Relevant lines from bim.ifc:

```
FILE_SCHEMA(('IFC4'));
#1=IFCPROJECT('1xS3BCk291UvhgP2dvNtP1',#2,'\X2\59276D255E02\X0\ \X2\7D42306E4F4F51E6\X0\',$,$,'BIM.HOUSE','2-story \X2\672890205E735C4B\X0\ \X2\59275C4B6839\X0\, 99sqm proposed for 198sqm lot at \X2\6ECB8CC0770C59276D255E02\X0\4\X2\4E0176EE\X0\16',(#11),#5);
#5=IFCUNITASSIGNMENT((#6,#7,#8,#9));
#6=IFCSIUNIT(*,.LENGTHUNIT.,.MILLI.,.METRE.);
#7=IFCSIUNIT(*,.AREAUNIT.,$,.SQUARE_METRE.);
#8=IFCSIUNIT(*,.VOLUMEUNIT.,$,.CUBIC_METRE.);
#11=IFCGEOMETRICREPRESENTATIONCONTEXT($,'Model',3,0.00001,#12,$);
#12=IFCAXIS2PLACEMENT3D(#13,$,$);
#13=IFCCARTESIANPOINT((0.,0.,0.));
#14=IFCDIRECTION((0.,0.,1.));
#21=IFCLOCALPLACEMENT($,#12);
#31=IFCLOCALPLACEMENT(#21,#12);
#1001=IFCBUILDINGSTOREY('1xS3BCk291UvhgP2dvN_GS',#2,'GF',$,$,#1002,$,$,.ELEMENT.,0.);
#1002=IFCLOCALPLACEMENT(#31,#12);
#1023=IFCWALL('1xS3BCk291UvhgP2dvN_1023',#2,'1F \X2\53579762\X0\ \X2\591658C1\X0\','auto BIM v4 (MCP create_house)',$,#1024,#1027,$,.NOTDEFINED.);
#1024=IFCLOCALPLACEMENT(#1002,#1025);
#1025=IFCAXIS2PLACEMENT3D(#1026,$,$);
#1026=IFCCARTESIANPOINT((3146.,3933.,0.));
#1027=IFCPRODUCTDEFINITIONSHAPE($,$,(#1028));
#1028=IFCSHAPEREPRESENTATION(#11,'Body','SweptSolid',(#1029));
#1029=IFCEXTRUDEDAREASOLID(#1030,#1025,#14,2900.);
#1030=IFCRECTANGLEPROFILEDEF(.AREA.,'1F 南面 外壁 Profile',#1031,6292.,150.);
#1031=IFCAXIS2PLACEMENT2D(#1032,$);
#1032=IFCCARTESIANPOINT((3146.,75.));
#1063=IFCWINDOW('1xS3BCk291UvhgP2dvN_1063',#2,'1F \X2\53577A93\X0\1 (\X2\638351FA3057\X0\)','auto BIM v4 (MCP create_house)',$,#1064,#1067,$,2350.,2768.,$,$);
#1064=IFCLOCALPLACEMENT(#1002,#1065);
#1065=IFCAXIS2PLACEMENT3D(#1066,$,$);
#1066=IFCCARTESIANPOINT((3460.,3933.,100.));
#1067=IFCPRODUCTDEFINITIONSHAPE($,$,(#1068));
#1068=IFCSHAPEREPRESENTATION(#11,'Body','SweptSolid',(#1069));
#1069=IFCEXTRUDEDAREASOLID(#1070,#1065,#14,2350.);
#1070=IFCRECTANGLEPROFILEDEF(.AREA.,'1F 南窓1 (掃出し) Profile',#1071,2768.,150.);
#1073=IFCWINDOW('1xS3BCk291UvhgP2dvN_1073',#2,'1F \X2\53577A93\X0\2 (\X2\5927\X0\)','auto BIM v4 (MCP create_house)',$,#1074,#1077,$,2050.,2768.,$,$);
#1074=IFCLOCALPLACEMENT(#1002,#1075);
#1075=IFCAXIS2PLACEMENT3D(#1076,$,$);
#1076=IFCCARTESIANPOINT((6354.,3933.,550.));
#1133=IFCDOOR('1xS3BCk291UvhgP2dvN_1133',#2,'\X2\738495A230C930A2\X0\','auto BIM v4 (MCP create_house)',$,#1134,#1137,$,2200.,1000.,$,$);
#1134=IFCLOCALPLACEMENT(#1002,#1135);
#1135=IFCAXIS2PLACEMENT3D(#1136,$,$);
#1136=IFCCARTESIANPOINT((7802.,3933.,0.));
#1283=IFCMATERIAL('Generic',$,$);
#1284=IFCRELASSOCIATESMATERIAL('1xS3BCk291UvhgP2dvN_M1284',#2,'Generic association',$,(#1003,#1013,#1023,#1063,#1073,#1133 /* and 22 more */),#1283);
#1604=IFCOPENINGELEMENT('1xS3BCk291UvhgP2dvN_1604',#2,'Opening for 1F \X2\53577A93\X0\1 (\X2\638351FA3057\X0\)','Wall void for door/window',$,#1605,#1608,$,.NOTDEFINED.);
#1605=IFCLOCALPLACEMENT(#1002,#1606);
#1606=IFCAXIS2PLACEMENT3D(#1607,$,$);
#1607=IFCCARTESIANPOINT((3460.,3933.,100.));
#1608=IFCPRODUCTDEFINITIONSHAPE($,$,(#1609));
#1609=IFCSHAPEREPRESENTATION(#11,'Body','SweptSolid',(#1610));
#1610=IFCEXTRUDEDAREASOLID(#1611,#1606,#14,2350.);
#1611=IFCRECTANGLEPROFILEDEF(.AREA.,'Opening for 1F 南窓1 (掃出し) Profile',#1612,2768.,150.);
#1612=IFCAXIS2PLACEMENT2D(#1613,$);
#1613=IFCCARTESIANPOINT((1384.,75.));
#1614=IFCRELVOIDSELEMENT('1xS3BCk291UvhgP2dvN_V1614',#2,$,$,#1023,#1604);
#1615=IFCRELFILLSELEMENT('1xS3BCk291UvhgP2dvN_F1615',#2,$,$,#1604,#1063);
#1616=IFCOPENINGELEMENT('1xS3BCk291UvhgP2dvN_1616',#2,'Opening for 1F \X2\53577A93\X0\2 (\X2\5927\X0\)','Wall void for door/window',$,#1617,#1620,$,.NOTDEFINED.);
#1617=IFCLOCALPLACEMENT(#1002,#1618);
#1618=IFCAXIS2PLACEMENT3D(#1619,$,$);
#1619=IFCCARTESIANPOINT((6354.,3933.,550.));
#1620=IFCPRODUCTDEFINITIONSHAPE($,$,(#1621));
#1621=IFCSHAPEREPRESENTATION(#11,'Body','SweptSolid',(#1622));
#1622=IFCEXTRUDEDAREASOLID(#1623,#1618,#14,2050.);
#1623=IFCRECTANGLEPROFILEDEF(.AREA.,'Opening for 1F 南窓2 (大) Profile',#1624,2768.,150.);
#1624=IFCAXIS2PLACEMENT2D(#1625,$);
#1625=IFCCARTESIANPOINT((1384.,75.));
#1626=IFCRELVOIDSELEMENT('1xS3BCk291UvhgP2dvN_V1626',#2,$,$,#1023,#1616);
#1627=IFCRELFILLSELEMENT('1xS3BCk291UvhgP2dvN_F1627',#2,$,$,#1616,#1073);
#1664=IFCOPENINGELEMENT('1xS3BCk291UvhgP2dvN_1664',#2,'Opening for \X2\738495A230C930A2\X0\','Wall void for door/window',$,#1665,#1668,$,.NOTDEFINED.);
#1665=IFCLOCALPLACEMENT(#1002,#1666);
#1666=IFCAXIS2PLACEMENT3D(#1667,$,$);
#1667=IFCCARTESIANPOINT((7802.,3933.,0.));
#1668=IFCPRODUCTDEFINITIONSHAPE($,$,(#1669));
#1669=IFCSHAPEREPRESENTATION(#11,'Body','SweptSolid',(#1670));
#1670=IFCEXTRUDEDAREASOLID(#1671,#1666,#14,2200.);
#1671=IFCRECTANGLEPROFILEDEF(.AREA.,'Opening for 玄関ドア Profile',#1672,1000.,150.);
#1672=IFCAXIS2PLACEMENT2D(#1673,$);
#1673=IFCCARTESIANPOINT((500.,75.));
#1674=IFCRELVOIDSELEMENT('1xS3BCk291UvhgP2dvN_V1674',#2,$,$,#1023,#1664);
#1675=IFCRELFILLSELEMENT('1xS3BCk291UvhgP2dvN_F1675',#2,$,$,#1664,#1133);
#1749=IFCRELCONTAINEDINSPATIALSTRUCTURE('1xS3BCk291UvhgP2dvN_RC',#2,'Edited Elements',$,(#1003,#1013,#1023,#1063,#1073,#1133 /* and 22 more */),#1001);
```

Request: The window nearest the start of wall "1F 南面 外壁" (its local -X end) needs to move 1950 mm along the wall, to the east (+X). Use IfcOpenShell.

```python
import ifcopenshell
import ifcopenshell.api.geometry
import ifcopenshell.util.placement
import ifcopenshell.util.unit

model = ifcopenshell.open("bim.ifc")
unit_scale = ifcopenshell.util.unit.calculate_unit_scale(model)

window = model.by_guid("1xS3BCk291UvhgP2dvN_1063")
opening = window.FillsVoids[0].RelatingOpeningElement
wall = opening.VoidsElements[0].RelatingBuildingElement

wall_matrix = ifcopenshell.util.placement.get_local_placement(wall.ObjectPlacement)
shift = wall_matrix[:3, 0] * 1.95 / unit_scale
before = ifcopenshell.util.placement.get_local_placement(window.ObjectPlacement)[:3, 3].copy()

# The window is not placed relative to its opening, so move both.
for product in (opening, window):
    matrix = ifcopenshell.util.placement.get_local_placement(product.ObjectPlacement)
    matrix[:3, 3] += shift
    ifcopenshell.api.geometry.edit_object_placement(model, product=product, matrix=matrix, is_si=False)

after = ifcopenshell.util.placement.get_local_placement(window.ObjectPlacement)[:3, 3]
print("window moved by", (after - before).round(3) + 0.0)

model.write("bim_rev.ifc")
```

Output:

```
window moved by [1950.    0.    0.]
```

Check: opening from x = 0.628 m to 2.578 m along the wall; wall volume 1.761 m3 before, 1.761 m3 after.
